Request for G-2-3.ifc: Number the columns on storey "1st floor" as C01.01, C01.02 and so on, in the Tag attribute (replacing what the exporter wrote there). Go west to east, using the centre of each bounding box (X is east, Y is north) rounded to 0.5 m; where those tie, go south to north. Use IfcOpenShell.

First a look at what the model holds.

```python
import ifcopenshell
import ifcopenshell.util.element
import ifcopenshell.util.placement

model = ifcopenshell.open("G-2-3.ifc")
print(model.schema)
storey = next(s for s in model.by_type("IfcBuildingStorey") if s.Name == "1st floor")
columns = [e for e in ifcopenshell.util.element.get_decomposition(storey) if e.is_a("IfcColumn")]
for e in sorted(columns, key=lambda e: e.id()):
    origin = ifcopenshell.util.placement.get_local_placement(e.ObjectPlacement)[:3, 3]
    print(e.id(), e.Tag, e.Name, origin.round(2) + 0.0, sep=" | ")
```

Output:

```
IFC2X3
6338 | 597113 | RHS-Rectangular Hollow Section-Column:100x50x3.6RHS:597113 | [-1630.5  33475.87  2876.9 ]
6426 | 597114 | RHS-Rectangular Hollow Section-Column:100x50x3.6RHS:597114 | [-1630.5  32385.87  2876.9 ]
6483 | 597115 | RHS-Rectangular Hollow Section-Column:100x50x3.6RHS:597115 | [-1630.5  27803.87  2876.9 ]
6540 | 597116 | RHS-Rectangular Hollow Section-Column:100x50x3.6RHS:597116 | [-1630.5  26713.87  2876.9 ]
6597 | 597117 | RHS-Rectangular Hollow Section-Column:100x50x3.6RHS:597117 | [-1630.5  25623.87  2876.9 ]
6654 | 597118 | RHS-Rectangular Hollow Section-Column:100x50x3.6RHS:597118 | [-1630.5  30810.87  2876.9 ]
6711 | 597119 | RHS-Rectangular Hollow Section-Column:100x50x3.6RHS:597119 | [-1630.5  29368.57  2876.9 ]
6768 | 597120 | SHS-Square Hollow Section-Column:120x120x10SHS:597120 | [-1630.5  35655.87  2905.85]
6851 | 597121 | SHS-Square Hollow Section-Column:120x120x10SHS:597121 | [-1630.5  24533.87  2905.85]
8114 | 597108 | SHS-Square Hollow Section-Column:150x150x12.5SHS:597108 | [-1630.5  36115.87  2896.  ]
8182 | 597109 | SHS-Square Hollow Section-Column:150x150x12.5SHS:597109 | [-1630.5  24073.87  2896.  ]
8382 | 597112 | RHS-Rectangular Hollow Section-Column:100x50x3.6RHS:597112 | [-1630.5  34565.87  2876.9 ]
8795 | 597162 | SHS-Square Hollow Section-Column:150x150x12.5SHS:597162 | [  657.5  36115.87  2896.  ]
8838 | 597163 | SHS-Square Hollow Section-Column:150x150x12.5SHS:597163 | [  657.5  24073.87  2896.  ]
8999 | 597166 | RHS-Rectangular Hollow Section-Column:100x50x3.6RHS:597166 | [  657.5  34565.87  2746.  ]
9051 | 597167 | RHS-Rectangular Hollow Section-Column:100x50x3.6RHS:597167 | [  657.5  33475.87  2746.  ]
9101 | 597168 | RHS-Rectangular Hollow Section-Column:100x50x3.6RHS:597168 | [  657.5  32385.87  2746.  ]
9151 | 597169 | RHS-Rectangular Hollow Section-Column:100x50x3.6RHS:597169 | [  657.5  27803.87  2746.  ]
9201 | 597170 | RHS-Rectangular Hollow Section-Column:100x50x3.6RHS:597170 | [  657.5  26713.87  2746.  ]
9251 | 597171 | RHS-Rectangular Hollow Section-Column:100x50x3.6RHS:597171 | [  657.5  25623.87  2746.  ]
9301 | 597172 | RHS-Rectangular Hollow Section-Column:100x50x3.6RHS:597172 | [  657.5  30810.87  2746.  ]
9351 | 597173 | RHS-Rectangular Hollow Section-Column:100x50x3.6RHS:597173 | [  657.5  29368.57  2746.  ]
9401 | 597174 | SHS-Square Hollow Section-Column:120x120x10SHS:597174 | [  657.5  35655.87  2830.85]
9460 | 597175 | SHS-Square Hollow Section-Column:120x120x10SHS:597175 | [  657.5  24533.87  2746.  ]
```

```python
import ifcopenshell
import ifcopenshell.geom
import ifcopenshell.util.element
import ifcopenshell.util.shape

model = ifcopenshell.open("G-2-3.ifc")
settings = ifcopenshell.geom.settings()
settings.set("use-world-coords", True)


def centre(element):
    shape = ifcopenshell.geom.create_shape(settings, element)
    return ifcopenshell.util.shape.get_bbox_centroid(shape.geometry)


storey = next(s for s in model.by_type("IfcBuildingStorey") if s.Name == "1st floor")
columns = [e for e in ifcopenshell.util.element.get_decomposition(storey) if e.is_a("IfcColumn")]

# Insertion points can sit at a corner or the storey origin, so sort by the geometry (in metres).
centres = {e: centre(e) for e in columns}
columns.sort(key=lambda e: (round(centres[e][0] / 0.5), centres[e][1]))

for i, e in enumerate(columns, start=1):
    number = f"C01.{i:02d}"
    e.Tag = number
    print(e.id(), number)

model.write("G-2-3_v2.ifc")
```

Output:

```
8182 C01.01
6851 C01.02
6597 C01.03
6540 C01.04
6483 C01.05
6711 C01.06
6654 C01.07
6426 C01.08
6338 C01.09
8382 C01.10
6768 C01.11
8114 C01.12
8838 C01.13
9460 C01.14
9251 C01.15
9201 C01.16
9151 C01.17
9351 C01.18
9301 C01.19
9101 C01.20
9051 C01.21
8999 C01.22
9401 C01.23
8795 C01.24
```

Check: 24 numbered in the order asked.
